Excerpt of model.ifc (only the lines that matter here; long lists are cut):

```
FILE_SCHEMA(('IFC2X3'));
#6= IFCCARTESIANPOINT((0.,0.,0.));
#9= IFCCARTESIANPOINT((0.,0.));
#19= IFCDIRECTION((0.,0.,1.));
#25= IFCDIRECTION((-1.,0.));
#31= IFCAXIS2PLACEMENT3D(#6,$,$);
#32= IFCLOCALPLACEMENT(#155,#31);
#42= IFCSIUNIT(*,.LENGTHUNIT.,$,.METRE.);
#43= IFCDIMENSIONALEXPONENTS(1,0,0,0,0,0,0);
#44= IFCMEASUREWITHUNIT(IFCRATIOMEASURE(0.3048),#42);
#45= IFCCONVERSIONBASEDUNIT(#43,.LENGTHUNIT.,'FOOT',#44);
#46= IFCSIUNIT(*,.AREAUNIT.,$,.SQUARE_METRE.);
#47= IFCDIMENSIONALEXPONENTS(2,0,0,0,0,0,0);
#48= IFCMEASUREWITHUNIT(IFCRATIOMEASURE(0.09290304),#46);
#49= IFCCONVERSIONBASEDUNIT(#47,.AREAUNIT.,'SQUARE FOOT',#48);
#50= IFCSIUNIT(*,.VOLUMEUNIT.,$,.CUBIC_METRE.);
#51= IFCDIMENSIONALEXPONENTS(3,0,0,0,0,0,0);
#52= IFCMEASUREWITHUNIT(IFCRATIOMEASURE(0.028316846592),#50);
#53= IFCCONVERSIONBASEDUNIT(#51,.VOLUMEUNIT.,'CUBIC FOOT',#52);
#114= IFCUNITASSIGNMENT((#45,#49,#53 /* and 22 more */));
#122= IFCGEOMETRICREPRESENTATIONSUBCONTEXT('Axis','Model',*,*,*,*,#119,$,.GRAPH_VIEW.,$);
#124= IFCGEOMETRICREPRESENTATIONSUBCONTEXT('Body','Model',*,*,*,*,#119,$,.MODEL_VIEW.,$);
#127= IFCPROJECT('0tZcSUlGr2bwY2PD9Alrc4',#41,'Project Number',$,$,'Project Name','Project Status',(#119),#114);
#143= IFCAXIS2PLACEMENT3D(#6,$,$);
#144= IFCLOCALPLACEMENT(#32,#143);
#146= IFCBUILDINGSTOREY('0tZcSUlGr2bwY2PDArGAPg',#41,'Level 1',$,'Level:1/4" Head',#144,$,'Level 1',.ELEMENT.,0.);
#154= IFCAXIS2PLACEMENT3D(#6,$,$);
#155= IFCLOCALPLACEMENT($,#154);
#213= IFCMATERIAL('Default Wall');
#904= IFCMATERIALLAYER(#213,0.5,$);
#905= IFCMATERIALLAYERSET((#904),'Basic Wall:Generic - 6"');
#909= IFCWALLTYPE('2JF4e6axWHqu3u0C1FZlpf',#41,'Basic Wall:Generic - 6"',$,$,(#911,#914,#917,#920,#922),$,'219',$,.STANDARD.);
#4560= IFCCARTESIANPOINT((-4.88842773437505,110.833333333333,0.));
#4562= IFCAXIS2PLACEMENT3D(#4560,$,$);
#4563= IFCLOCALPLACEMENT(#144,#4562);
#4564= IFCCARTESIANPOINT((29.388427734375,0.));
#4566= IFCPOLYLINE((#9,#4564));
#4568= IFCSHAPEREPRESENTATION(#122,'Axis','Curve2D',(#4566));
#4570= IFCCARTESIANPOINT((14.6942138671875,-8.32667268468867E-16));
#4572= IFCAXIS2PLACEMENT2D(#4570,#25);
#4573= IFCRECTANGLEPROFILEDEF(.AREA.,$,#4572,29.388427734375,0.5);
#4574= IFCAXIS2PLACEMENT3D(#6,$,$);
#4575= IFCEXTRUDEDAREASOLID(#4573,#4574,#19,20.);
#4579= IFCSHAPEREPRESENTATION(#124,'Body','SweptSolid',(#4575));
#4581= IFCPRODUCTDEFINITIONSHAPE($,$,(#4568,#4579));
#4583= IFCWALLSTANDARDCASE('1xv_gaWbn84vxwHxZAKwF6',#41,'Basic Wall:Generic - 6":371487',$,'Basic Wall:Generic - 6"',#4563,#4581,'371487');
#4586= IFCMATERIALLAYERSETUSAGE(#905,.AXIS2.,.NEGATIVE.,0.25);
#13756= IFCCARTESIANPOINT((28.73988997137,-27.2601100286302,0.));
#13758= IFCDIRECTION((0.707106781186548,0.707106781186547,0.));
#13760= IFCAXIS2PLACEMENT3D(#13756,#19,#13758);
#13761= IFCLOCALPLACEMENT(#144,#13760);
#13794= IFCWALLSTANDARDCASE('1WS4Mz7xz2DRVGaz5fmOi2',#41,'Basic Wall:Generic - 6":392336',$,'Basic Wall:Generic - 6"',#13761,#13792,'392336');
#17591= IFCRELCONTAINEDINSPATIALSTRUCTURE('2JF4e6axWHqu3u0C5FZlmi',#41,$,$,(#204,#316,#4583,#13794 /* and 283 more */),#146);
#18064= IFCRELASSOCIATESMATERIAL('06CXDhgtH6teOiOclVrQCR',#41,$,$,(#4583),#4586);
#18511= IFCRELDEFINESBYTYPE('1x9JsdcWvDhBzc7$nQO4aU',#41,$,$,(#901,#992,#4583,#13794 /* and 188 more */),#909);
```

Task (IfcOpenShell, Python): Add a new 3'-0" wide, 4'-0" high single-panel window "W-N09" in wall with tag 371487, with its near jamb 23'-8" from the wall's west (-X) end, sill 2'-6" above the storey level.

```python
import numpy as np
import ifcopenshell
import ifcopenshell.api.feature
import ifcopenshell.api.geometry
import ifcopenshell.api.root
import ifcopenshell.api.spatial
import ifcopenshell.api.type
import ifcopenshell.geom
import ifcopenshell.util.element
import ifcopenshell.util.placement
import ifcopenshell.util.representation
import ifcopenshell.util.shape
import ifcopenshell.util.unit

model = ifcopenshell.open("model.ifc")
unit_scale = ifcopenshell.util.unit.calculate_unit_scale(model)
settings = ifcopenshell.geom.settings()


def volume(element):
    """Net volume in cubic metres, openings subtracted."""
    shape = ifcopenshell.geom.create_shape(settings, element)
    return ifcopenshell.util.shape.get_volume(shape.geometry)


wall = model.by_guid("1xv_gaWbn84vxwHxZAKwF6")
storey = ifcopenshell.util.element.get_container(wall, ifc_class="IfcBuildingStorey")
context = ifcopenshell.util.representation.get_context(model, "Model", "Body", "MODEL_VIEW")
before = volume(wall)

width, height, from_end, sill = 0.9144, 1.2192, 7.2136, 0.762  # metres

# The wall runs along its own X axis, and the end named is its -X end.
wall_shape = ifcopenshell.geom.create_shape(settings, wall)
x, y, z = ifcopenshell.util.shape.get_vertices(wall_shape.geometry).T
start = x.min() + from_end
face, thickness = float(y.min()), float(y.max() - y.min())
wall_matrix = ifcopenshell.util.placement.get_local_placement(wall.ObjectPlacement)
level = ifcopenshell.util.placement.get_local_placement(storey.ObjectPlacement)[2, 3]


def in_wall(x, y):
    """Placement at x, y metres in the wall's axes, at sill height."""
    matrix = wall_matrix.copy()
    matrix[:, 3] = wall_matrix @ np.array([x / unit_scale, y / unit_scale, 0.0, 1.0])
    matrix[2, 3] = level + sill / unit_scale
    return matrix


# Opening: a box that overshoots both wall faces by 50 mm.
opening = ifcopenshell.api.root.create_entity(model, ifc_class="IfcOpeningElement")
box = ifcopenshell.api.geometry.add_wall_representation(
    model, context=context, length=width, height=height, thickness=thickness + 0.1
)
ifcopenshell.api.geometry.assign_representation(model, product=opening, representation=box)
ifcopenshell.api.geometry.edit_object_placement(model, product=opening, matrix=in_wall(start, face - 0.05), is_si=False)
ifcopenshell.api.feature.add_feature(model, feature=opening, element=wall)

window = ifcopenshell.api.root.create_entity(model, ifc_class="IfcWindow", name="W-N09")
window.OverallWidth, window.OverallHeight = width / unit_scale, height / unit_scale
body = ifcopenshell.api.geometry.add_window_representation(
    model,
    context=context,
    overall_width=window.OverallWidth,
    overall_height=window.OverallHeight,
    partition_type="SINGLE_PANEL",
)
ifcopenshell.api.geometry.assign_representation(model, product=window, representation=body)
ifcopenshell.api.spatial.assign_container(model, products=[window], relating_structure=storey)
fills = ifcopenshell.api.feature.add_filling(model, opening=opening, element=window)
fills.OwnerHistory = window.OwnerHistory  # required in IFC2X3

# IFC2X3 keeps the operation on the window style.
style = ifcopenshell.api.root.create_entity(model, ifc_class="IfcWindowStyle", name="W-N09")
style.OperationType, style.ConstructionType = "SINGLE_PANEL", "NOTDEFINED"
style.ParameterTakesPrecedence = style.Sizeable = False
ifcopenshell.api.type.assign_type(model, related_objects=[window], relating_type=style)

# Centre the window in the wall's thickness.
ifcopenshell.api.geometry.edit_object_placement(model, product=window, matrix=in_wall(start, face), is_si=False)
window_shape = ifcopenshell.geom.create_shape(settings, window)
depth = ifcopenshell.util.shape.get_vertices(window_shape.geometry)[:, 1]
offset = face + thickness / 2 - (depth.min() + depth.max()) / 2
ifcopenshell.api.geometry.edit_object_placement(model, product=window, matrix=in_wall(start, offset), is_si=False)

after = volume(wall)

print(f"wall volume {before:.3f} -> {after:.3f} m3")

model.write("model_updated.ifc")
```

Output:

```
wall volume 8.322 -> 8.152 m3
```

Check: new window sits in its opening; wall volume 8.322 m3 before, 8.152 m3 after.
